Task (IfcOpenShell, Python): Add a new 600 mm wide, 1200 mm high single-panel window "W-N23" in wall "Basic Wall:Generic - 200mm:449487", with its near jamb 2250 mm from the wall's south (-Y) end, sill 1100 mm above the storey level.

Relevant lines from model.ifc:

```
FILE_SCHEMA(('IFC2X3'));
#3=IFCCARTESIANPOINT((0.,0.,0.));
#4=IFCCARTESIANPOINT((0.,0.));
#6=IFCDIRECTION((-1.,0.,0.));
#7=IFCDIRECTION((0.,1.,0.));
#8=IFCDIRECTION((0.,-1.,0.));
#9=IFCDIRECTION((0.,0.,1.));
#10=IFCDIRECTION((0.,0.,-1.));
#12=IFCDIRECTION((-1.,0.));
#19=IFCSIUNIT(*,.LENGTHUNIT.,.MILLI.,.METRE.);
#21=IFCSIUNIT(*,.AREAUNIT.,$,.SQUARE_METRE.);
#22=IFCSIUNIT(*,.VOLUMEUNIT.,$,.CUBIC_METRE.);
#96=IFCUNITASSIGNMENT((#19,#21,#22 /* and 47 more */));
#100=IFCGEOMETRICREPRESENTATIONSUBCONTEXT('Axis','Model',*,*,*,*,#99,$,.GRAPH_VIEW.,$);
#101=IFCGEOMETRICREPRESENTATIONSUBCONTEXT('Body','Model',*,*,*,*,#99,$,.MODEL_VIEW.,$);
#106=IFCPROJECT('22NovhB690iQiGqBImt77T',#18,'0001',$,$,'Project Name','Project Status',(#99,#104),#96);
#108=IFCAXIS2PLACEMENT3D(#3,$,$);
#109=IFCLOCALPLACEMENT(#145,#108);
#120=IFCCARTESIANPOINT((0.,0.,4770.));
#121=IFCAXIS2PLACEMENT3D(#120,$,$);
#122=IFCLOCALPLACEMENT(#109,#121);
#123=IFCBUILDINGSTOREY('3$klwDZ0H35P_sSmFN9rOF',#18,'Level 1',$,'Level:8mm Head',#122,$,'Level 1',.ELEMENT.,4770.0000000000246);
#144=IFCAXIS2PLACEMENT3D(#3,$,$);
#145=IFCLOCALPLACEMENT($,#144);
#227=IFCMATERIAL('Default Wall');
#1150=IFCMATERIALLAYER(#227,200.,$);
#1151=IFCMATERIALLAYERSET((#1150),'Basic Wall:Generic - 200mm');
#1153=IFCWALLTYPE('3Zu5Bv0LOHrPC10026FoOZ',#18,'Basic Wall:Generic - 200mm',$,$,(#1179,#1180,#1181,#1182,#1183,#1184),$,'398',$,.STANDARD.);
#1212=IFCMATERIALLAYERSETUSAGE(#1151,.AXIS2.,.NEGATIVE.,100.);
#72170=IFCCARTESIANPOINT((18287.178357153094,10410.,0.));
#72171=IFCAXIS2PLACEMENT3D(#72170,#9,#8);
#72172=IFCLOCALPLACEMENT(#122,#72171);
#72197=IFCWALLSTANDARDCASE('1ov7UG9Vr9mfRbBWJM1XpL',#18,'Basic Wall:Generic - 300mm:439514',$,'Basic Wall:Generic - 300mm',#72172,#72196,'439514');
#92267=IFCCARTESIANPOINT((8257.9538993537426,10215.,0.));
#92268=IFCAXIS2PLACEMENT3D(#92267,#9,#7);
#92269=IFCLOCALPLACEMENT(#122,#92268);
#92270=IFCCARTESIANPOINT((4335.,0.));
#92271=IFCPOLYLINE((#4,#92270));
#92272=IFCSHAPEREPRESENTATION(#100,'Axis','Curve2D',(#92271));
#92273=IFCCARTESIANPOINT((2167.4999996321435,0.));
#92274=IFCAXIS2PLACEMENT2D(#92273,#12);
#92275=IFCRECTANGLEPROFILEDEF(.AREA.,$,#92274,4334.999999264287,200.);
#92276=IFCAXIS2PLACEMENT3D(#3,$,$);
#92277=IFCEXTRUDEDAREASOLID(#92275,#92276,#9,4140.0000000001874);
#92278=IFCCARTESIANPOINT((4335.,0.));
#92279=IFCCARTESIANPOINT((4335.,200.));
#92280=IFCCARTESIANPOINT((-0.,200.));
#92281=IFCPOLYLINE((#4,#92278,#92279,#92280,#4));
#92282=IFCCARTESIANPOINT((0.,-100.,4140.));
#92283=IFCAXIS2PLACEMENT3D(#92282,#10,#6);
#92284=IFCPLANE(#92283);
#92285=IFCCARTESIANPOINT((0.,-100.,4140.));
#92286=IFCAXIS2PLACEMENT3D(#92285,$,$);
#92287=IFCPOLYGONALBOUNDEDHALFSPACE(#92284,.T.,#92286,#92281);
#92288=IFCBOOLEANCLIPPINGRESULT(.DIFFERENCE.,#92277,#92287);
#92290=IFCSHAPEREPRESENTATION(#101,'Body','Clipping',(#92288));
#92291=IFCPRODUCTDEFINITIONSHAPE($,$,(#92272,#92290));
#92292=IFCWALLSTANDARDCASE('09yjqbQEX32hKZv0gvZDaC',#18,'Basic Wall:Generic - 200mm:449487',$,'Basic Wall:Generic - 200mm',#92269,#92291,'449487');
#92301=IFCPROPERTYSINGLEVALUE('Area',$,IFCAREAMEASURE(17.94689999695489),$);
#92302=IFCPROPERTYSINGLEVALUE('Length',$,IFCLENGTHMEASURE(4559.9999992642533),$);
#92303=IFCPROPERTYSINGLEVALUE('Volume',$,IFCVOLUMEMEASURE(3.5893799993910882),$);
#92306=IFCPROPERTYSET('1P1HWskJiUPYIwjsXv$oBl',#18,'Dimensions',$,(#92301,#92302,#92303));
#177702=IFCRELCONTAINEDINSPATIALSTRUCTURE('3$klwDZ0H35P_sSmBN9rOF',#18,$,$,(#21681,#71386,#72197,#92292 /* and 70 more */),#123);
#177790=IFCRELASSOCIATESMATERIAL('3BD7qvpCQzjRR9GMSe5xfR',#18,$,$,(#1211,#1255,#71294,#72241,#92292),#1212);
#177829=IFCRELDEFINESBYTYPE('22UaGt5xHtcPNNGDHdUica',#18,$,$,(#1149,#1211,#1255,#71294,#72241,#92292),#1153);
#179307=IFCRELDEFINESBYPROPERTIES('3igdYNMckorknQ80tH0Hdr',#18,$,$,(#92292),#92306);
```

```python
import numpy as np
import ifcopenshell
import ifcopenshell.api.feature
import ifcopenshell.api.geometry
import ifcopenshell.api.pset
import ifcopenshell.api.root
import ifcopenshell.api.spatial
import ifcopenshell.api.type
import ifcopenshell.geom
import ifcopenshell.util.element
import ifcopenshell.util.placement
import ifcopenshell.util.representation
import ifcopenshell.util.shape
import ifcopenshell.util.unit

model = ifcopenshell.open("model.ifc")
unit_scale = ifcopenshell.util.unit.calculate_unit_scale(model)
area_scale = ifcopenshell.util.unit.calculate_unit_scale(model, "AREAUNIT")
volume_scale = ifcopenshell.util.unit.calculate_unit_scale(model, "VOLUMEUNIT")
settings = ifcopenshell.geom.settings()


def volume(element):
    """Net volume in cubic metres, openings subtracted."""
    shape = ifcopenshell.geom.create_shape(settings, element)
    return ifcopenshell.util.shape.get_volume(shape.geometry)


wall = model.by_guid("09yjqbQEX32hKZv0gvZDaC")
storey = ifcopenshell.util.element.get_container(wall, ifc_class="IfcBuildingStorey")
context = ifcopenshell.util.representation.get_context(model, "Model", "Body", "MODEL_VIEW")
before = volume(wall)

width, height, from_end, sill = 0.6, 1.2, 2.25, 1.1  # metres

# The wall runs along its own X axis, and the end named is its -X end.
wall_shape = ifcopenshell.geom.create_shape(settings, wall)
x, y, z = ifcopenshell.util.shape.get_vertices(wall_shape.geometry).T
start = x.min() + from_end
face, thickness = float(y.min()), float(y.max() - y.min())
wall_matrix = ifcopenshell.util.placement.get_local_placement(wall.ObjectPlacement)
level = ifcopenshell.util.placement.get_local_placement(storey.ObjectPlacement)[2, 3]


def in_wall(x, y):
    """Placement at x, y metres in the wall's axes, at sill height."""
    matrix = wall_matrix.copy()
    matrix[:, 3] = wall_matrix @ np.array([x / unit_scale, y / unit_scale, 0.0, 1.0])
    matrix[2, 3] = level + sill / unit_scale
    return matrix


# Opening: a box that overshoots both wall faces by 50 mm.
opening = ifcopenshell.api.root.create_entity(model, ifc_class="IfcOpeningElement")
box = ifcopenshell.api.geometry.add_wall_representation(
    model, context=context, length=width, height=height, thickness=thickness + 0.1
)
ifcopenshell.api.geometry.assign_representation(model, product=opening, representation=box)
ifcopenshell.api.geometry.edit_object_placement(model, product=opening, matrix=in_wall(start, face - 0.05), is_si=False)
ifcopenshell.api.feature.add_feature(model, feature=opening, element=wall)

window = ifcopenshell.api.root.create_entity(model, ifc_class="IfcWindow", name="W-N23")
window.OverallWidth, window.OverallHeight = width / unit_scale, height / unit_scale
body = ifcopenshell.api.geometry.add_window_representation(
    model,
    context=context,
    overall_width=window.OverallWidth,
    overall_height=window.OverallHeight,
    partition_type="SINGLE_PANEL",
)
ifcopenshell.api.geometry.assign_representation(model, product=window, representation=body)
ifcopenshell.api.spatial.assign_container(model, products=[window], relating_structure=storey)
fills = ifcopenshell.api.feature.add_filling(model, opening=opening, element=window)
fills.OwnerHistory = window.OwnerHistory  # required in IFC2X3

# IFC2X3 keeps the operation on the window style.
style = ifcopenshell.api.root.create_entity(model, ifc_class="IfcWindowStyle", name="W-N23")
style.OperationType, style.ConstructionType = "SINGLE_PANEL", "NOTDEFINED"
style.ParameterTakesPrecedence = style.Sizeable = False
ifcopenshell.api.type.assign_type(model, related_objects=[window], relating_type=style)

# Centre the window in the wall's thickness.
ifcopenshell.api.geometry.edit_object_placement(model, product=window, matrix=in_wall(start, face), is_si=False)
window_shape = ifcopenshell.geom.create_shape(settings, window)
depth = ifcopenshell.util.shape.get_vertices(window_shape.geometry)[:, 1]
offset = face + thickness / 2 - (depth.min() + depth.max()) / 2
ifcopenshell.api.geometry.edit_object_placement(model, product=window, matrix=in_wall(start, offset), is_si=False)

after = volume(wall)

# Update the wall's stored quantities.
pset = model.by_id(ifcopenshell.util.element.get_pset(wall, "Dimensions", should_inherit=False)["id"])
ifcopenshell.api.pset.edit_pset(model, pset=pset, properties={
    "Area": model.create_entity("IfcAreaMeasure", after / thickness / area_scale),
    "Volume": model.create_entity("IfcVolumeMeasure", after / volume_scale),
})

print(f"wall volume {before:.3f} -> {after:.3f} m3")

model.write("model_updated.ifc")
```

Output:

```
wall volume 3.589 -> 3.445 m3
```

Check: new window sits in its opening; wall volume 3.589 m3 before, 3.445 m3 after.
